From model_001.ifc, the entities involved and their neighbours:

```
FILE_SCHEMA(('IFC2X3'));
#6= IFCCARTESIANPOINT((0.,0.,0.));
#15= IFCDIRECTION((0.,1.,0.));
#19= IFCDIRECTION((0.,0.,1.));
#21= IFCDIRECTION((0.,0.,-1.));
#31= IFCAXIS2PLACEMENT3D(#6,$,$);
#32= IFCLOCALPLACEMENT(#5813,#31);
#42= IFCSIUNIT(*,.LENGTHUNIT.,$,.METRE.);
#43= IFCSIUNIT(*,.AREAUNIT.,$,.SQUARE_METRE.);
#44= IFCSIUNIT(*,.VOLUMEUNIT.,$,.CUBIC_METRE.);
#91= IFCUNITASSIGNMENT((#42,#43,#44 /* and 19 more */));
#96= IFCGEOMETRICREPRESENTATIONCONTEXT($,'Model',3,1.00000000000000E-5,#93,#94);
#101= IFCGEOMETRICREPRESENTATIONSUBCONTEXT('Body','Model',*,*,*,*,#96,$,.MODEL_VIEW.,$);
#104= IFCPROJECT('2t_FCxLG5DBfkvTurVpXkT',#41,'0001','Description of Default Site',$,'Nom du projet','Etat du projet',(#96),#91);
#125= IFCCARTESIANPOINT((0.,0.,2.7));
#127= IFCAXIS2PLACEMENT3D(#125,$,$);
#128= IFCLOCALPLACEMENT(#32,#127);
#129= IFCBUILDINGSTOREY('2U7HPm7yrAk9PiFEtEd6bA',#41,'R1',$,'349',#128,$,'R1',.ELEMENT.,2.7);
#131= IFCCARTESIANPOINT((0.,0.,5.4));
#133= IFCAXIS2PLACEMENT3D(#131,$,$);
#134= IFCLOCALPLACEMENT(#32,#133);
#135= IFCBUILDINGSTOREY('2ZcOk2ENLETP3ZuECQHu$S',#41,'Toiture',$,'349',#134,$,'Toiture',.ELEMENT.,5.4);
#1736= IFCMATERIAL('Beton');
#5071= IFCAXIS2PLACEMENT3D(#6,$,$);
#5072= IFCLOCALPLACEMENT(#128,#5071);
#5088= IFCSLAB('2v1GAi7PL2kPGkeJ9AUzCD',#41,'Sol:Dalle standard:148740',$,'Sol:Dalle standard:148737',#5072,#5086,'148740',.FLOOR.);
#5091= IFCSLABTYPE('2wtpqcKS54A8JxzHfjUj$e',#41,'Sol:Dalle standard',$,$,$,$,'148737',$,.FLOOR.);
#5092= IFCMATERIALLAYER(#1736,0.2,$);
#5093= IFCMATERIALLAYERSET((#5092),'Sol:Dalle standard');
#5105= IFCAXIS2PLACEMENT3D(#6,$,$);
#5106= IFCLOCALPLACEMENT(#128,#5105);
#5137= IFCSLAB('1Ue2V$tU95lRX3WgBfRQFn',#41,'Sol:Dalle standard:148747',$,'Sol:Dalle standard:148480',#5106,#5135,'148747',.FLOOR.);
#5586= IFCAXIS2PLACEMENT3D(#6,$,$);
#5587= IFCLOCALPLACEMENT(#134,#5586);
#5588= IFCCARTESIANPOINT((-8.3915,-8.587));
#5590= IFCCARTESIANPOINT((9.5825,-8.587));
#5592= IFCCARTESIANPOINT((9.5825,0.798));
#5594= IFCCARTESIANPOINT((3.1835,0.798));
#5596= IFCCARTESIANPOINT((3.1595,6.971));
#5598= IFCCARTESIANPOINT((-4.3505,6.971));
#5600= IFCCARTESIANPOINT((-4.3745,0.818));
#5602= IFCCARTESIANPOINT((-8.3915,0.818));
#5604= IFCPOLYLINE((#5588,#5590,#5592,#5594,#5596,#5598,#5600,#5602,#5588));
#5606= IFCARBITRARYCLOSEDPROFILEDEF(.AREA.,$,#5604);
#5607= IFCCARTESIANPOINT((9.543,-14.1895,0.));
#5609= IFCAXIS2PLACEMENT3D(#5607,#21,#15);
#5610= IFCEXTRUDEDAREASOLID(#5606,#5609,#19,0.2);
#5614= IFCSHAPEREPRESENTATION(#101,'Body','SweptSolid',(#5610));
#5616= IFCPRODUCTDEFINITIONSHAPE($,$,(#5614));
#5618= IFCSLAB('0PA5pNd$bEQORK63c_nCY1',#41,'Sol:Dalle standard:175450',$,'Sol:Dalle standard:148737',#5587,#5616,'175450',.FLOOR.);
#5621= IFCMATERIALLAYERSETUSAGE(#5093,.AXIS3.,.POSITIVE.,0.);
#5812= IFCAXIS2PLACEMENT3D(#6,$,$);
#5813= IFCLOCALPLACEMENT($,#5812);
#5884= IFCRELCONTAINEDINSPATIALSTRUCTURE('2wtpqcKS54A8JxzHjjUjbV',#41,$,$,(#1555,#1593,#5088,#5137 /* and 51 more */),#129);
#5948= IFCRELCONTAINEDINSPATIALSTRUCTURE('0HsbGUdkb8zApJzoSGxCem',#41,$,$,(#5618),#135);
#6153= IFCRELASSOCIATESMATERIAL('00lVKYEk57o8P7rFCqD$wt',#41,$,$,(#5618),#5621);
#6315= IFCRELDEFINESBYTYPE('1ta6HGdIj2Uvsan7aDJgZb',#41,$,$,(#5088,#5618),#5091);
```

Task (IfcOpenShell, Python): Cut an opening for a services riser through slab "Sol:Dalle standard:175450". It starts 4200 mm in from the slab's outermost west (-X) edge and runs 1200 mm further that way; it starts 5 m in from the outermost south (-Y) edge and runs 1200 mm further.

```python
import numpy as np
import ifcopenshell
import ifcopenshell.api.feature
import ifcopenshell.api.geometry
import ifcopenshell.api.root
import ifcopenshell.geom
import ifcopenshell.util.placement
import ifcopenshell.util.representation
import ifcopenshell.util.shape
import ifcopenshell.util.unit

model = ifcopenshell.open("model_001.ifc")
unit_scale = ifcopenshell.util.unit.calculate_unit_scale(model)
settings = ifcopenshell.geom.settings()


def volume(element):
    """Net volume in cubic metres, openings subtracted."""
    shape = ifcopenshell.geom.create_shape(settings, element)
    return ifcopenshell.util.shape.get_volume(shape.geometry)


slab = model.by_guid("0PA5pNd$bEQORK63c_nCY1")
before = volume(slab)

# Extent in the slab's own axes, in metres. The edges named are its -X and -Y sides.
slab_shape = ifcopenshell.geom.create_shape(settings, slab)
vertices = ifcopenshell.util.shape.get_vertices(slab_shape.geometry)
x_min, y_min, bottom = vertices.min(axis=0)
top = vertices[:, 2].max()

opening = ifcopenshell.api.root.create_entity(model, ifc_class="IfcOpeningElement", name="Services riser opening")
context = ifcopenshell.util.representation.get_context(model, "Model", "Body", "MODEL_VIEW")
width, depth = 1.2, 1.2
outline = [(0.0, 0.0), (width, 0.0), (width, depth), (0.0, depth), (0.0, 0.0)]
# Overshoot both faces by 50 mm so the cut is clean.
shape = ifcopenshell.api.geometry.add_slab_representation(
    model, context=context, depth=top - bottom + 0.1, polyline=outline
)
ifcopenshell.api.geometry.assign_representation(model, product=opening, representation=shape)

matrix = ifcopenshell.util.placement.get_local_placement(slab.ObjectPlacement)
matrix[:, 3] = matrix @ np.append(np.array([x_min + 4.2, y_min + 5, bottom - 0.05]) / unit_scale, 1.0)
ifcopenshell.api.geometry.edit_object_placement(model, product=opening, matrix=matrix, is_si=False)
ifcopenshell.api.feature.add_feature(model, feature=opening, element=slab)

after = volume(slab)

print(f"slab volume {before:.3f} -> {after:.3f} m3")

model.write("model_001-out.ifc")
```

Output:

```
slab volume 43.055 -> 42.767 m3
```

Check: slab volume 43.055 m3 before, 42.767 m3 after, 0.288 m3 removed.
